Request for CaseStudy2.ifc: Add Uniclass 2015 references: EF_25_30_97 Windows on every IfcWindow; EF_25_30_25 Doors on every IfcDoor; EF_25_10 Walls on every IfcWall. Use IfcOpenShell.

First a look at what the model holds.

```python
import ifcopenshell

model = ifcopenshell.open("CaseStudy2.ifc")
print(model.schema)
print("classifications:", [c.Name for c in model.by_type("IfcClassification")])
for ifc_class in ("IfcDoor", "IfcRoof", "IfcStair", "IfcWall", "IfcWindow"):
    print(ifc_class, len(model.by_type(ifc_class)))
```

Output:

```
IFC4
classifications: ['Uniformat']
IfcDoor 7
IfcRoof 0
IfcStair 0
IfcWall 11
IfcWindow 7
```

```python
import ifcopenshell
import ifcopenshell.api.classification

model = ifcopenshell.open("CaseStudy2.ifc")

system = ifcopenshell.api.classification.add_classification(model, classification="Uniclass 2015")

codes = {
    "IfcWindow": ("EF_25_30_97", "Windows"),
    "IfcDoor": ("EF_25_30_25", "Doors"),
    "IfcWall": ("EF_25_10", "Walls"),
}
for ifc_class, (code, name) in codes.items():
    products = model.by_type(ifc_class)
    ifcopenshell.api.classification.add_reference(
        model, products=products, classification=system, identification=code, name=name
    )
    print(code, len(products))

model.write("CaseStudy2-out.ifc")
```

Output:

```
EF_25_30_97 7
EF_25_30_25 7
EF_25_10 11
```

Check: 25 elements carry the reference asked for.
